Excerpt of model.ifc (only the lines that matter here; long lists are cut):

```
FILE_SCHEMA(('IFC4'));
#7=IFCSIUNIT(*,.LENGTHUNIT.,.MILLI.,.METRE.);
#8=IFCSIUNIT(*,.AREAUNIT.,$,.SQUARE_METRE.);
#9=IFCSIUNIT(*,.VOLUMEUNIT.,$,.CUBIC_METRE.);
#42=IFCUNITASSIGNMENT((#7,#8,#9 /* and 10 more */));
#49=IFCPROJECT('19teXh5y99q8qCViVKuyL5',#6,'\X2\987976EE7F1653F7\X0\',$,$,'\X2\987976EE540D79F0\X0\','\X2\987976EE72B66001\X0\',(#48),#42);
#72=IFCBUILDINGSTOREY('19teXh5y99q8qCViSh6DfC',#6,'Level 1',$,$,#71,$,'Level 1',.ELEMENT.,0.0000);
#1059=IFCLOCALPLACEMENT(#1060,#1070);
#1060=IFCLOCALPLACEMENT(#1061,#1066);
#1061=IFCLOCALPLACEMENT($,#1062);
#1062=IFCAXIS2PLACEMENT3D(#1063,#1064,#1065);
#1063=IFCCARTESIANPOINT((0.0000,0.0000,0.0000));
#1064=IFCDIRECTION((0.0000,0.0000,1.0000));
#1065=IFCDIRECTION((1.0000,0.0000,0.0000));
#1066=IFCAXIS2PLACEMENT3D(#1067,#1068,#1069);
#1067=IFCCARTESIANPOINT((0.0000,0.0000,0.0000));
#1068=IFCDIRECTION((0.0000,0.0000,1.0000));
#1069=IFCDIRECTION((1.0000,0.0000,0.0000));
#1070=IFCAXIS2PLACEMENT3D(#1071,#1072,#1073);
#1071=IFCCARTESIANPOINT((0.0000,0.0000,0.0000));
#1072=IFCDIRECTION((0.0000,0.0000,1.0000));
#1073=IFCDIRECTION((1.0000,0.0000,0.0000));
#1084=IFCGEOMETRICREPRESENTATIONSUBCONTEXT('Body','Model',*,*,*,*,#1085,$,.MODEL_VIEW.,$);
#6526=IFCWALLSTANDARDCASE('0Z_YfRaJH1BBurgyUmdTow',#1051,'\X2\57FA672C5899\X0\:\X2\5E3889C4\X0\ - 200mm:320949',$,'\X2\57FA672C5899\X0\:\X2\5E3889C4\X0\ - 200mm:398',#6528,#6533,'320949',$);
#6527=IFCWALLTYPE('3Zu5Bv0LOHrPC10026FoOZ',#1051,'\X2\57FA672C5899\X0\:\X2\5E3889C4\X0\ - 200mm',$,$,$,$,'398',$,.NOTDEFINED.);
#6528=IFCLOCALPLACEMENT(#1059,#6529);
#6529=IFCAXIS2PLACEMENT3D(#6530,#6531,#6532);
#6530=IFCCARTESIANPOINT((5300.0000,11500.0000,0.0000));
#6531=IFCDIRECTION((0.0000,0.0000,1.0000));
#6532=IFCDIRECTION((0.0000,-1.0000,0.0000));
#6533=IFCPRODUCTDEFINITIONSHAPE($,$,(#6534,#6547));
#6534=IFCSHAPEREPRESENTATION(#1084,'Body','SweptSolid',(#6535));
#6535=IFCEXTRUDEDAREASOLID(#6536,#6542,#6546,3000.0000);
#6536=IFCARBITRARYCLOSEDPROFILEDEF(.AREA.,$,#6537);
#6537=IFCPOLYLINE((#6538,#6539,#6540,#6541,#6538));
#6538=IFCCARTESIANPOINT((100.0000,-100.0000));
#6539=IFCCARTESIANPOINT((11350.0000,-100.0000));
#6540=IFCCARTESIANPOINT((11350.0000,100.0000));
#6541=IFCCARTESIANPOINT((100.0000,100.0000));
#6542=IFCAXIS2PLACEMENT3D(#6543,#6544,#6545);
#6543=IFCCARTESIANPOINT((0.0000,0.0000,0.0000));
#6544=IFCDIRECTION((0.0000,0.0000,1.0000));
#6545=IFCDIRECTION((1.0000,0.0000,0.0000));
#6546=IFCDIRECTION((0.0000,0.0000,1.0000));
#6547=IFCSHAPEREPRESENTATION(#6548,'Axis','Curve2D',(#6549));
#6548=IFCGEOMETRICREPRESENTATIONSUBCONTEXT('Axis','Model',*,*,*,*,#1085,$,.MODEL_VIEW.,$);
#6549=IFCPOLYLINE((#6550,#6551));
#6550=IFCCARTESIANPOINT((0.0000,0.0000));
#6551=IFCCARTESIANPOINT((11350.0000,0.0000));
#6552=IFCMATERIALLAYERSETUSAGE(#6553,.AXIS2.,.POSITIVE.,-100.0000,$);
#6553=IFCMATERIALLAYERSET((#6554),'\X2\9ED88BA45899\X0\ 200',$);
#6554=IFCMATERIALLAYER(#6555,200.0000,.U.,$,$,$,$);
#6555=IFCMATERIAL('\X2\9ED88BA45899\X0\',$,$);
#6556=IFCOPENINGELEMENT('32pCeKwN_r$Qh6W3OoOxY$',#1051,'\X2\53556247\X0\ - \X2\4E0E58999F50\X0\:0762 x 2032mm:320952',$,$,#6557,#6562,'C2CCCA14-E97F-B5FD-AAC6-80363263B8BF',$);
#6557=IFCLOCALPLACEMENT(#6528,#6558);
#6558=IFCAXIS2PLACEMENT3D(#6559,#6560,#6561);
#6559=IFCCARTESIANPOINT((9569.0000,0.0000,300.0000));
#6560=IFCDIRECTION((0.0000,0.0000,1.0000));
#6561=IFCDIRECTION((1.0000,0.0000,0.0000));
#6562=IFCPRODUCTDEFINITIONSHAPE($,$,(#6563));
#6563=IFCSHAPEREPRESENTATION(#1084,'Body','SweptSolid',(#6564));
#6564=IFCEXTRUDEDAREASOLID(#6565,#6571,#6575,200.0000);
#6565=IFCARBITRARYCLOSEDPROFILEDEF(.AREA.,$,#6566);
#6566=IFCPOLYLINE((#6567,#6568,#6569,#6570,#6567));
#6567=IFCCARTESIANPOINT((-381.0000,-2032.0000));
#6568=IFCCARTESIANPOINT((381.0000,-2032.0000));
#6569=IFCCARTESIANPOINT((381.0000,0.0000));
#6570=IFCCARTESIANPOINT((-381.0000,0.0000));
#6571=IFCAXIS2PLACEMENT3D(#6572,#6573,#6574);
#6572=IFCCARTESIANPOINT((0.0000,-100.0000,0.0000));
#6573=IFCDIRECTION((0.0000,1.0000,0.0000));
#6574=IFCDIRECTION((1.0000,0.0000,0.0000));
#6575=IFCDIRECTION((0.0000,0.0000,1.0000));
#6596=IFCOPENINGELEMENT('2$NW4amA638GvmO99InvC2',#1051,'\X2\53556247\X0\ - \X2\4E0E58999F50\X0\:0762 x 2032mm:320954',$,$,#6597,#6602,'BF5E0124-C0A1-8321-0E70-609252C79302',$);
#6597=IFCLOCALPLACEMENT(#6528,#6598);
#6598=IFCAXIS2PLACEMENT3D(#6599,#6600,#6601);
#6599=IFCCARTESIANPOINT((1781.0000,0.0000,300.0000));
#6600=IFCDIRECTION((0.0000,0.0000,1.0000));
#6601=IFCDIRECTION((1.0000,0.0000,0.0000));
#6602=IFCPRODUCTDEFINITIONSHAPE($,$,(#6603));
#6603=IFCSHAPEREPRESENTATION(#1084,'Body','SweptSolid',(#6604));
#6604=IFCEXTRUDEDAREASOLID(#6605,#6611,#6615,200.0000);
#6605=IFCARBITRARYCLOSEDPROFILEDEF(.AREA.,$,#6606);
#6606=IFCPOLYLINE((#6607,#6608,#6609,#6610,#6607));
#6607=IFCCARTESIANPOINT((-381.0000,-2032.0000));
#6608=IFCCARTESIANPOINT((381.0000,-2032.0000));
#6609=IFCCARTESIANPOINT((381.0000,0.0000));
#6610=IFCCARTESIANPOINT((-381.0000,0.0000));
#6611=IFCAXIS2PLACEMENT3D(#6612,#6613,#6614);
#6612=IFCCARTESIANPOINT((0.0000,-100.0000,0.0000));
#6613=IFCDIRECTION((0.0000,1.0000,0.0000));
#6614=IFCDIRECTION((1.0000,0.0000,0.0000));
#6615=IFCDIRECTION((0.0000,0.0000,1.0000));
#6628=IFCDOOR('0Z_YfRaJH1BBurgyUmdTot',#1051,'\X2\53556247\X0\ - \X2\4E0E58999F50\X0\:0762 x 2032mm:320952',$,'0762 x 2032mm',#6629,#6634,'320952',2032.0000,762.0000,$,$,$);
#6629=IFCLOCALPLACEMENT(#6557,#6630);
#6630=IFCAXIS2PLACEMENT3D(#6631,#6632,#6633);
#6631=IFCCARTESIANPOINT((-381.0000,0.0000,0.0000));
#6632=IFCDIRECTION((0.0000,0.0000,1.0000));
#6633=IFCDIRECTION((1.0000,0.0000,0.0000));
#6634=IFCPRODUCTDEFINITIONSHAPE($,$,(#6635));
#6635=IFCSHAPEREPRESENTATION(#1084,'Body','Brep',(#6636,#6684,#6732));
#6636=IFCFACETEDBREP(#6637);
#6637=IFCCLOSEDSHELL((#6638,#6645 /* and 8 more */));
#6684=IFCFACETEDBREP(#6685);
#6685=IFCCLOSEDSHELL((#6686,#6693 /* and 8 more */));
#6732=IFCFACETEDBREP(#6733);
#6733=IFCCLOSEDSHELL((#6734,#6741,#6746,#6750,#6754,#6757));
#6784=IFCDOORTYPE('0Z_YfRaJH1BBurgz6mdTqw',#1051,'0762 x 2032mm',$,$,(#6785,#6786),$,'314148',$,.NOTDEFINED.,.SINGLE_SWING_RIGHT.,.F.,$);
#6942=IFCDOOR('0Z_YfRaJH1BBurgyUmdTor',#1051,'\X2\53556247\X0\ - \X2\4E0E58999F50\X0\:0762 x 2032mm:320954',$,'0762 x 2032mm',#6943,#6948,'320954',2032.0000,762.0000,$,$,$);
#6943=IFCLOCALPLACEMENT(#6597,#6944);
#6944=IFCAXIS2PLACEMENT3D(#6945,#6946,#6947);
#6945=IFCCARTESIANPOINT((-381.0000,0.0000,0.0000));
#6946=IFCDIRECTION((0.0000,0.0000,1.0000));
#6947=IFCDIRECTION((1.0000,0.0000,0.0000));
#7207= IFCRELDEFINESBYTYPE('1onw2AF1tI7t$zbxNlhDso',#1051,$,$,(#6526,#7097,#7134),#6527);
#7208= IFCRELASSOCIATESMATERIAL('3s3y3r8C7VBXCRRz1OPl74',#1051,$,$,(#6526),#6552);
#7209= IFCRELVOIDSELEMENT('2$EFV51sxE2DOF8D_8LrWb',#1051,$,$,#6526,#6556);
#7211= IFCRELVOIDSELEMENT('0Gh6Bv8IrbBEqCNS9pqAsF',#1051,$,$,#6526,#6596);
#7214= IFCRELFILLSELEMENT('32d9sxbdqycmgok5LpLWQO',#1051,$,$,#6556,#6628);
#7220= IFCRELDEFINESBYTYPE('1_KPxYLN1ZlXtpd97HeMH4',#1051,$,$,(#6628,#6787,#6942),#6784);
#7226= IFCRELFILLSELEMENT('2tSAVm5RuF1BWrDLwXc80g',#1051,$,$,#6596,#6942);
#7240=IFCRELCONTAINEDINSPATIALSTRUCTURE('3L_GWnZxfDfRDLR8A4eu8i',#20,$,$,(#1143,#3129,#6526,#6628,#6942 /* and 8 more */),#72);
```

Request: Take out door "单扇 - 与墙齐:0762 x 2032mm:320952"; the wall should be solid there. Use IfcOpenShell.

```python
import ifcopenshell
import ifcopenshell.api.feature
import ifcopenshell.api.root
import ifcopenshell.geom
import ifcopenshell.util.shape

model = ifcopenshell.open("model.ifc")
settings = ifcopenshell.geom.settings()


def volume(element):
    """Net volume in cubic metres, openings subtracted."""
    shape = ifcopenshell.geom.create_shape(settings, element)
    return ifcopenshell.util.shape.get_volume(shape.geometry)


door = model.by_guid("0Z_YfRaJH1BBurgyUmdTot")
opening = door.FillsVoids[0].RelatingOpeningElement
wall = opening.VoidsElements[0].RelatingBuildingElement
before = volume(wall)

ifcopenshell.api.root.remove_product(model, product=door)
ifcopenshell.api.feature.remove_feature(model, feature=opening)

after = volume(wall)

print(f"wall volume {before:.3f} -> {after:.3f} m3")

model.write("model_rev.ifc")
```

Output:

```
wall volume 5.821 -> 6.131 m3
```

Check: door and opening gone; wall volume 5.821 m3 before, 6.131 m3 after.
